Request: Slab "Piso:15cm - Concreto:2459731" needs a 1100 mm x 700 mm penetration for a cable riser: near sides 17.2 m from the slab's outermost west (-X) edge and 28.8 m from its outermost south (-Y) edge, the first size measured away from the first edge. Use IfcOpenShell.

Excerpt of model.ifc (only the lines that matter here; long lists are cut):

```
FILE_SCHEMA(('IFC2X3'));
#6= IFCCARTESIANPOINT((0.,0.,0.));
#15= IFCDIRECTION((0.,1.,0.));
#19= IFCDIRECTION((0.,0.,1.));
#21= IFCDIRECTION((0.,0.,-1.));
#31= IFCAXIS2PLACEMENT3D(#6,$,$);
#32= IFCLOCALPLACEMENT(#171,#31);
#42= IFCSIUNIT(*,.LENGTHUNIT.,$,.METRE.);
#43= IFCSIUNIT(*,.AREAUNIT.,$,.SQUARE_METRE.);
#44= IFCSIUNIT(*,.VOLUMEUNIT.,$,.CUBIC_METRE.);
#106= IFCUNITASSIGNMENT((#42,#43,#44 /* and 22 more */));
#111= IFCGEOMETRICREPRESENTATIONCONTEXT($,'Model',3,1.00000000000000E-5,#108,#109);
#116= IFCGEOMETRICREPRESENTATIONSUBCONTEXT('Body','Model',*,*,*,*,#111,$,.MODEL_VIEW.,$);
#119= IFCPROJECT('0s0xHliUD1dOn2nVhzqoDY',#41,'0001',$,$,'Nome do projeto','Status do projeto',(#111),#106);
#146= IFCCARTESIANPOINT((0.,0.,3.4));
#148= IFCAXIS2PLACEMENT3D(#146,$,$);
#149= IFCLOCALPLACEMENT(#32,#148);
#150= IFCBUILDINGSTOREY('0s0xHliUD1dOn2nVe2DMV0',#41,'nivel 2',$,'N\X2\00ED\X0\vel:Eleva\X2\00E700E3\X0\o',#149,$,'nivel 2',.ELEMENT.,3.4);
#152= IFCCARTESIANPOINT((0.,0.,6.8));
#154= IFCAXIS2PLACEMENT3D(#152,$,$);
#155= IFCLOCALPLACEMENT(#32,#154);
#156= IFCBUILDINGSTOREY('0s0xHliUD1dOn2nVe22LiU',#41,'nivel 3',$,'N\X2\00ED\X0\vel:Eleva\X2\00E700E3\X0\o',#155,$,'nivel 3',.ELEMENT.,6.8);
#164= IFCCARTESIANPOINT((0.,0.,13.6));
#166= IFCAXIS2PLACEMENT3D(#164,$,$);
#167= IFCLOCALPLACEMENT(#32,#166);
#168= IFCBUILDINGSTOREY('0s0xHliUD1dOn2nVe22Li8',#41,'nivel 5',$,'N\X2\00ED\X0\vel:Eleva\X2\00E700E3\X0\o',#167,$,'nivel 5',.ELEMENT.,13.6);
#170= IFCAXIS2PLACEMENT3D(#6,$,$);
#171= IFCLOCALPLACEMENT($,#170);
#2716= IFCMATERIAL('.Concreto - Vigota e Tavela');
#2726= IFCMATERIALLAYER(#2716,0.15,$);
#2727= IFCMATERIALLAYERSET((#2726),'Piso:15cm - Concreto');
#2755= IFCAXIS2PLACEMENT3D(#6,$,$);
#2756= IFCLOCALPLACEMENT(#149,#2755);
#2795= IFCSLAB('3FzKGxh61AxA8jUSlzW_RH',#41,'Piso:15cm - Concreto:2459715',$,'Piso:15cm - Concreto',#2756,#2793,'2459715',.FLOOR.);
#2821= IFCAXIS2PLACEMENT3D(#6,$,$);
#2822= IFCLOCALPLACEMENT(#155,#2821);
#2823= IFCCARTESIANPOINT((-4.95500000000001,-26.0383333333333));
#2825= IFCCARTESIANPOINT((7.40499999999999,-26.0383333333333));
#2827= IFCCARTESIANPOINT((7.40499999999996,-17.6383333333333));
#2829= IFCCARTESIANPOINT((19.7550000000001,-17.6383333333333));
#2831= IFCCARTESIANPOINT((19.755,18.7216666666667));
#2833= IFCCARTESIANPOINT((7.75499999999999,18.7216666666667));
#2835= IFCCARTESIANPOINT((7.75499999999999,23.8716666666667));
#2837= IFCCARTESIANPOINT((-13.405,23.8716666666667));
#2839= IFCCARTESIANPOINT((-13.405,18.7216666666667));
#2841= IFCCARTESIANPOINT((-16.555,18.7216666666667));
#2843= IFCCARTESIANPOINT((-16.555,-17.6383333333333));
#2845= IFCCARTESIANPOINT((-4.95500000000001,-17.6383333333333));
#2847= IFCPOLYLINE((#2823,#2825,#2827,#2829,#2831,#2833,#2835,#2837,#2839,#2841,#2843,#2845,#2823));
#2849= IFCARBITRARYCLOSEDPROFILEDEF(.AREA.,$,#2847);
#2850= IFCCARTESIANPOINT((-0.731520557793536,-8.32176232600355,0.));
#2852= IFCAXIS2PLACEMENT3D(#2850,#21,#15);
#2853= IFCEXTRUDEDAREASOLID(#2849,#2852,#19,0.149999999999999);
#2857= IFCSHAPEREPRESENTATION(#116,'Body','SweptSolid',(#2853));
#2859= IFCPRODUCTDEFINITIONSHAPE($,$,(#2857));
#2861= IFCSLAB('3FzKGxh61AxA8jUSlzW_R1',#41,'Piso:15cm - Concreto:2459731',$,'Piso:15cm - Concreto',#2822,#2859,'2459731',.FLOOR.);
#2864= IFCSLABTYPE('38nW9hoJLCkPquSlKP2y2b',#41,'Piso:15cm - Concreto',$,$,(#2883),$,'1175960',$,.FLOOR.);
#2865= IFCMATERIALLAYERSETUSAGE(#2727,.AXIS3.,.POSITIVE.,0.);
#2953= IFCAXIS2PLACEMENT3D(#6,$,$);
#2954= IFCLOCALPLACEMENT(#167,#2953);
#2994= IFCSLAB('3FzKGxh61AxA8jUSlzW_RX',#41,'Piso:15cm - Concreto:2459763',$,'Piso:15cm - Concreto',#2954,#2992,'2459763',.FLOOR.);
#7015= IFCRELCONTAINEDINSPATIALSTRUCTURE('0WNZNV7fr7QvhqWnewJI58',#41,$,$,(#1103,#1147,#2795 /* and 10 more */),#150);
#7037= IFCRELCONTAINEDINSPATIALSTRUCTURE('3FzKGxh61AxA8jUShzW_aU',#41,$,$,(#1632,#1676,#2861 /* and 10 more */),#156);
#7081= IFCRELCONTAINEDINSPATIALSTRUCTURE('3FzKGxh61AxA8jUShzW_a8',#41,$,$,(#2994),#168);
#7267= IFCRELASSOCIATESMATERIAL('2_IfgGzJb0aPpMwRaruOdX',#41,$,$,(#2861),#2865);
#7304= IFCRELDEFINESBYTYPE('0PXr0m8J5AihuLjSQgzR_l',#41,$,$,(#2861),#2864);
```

```python
import numpy as np
import ifcopenshell
import ifcopenshell.api.feature
import ifcopenshell.api.geometry
import ifcopenshell.api.root
import ifcopenshell.geom
import ifcopenshell.util.placement
import ifcopenshell.util.representation
import ifcopenshell.util.shape
import ifcopenshell.util.unit

model = ifcopenshell.open("model.ifc")
unit_scale = ifcopenshell.util.unit.calculate_unit_scale(model)
settings = ifcopenshell.geom.settings()


def volume(element):
    """Net volume in cubic metres, openings subtracted."""
    shape = ifcopenshell.geom.create_shape(settings, element)
    return ifcopenshell.util.shape.get_volume(shape.geometry)


slab = model.by_guid("3FzKGxh61AxA8jUSlzW_R1")
before = volume(slab)

# Extent in the slab's own axes, in metres. The edges named are its -X and -Y sides.
slab_shape = ifcopenshell.geom.create_shape(settings, slab)
vertices = ifcopenshell.util.shape.get_vertices(slab_shape.geometry)
x_min, y_min, bottom = vertices.min(axis=0)
top = vertices[:, 2].max()

opening = ifcopenshell.api.root.create_entity(model, ifc_class="IfcOpeningElement", name="Cable riser opening")
context = ifcopenshell.util.representation.get_context(model, "Model", "Body", "MODEL_VIEW")
width, depth = 1.1, 0.7
outline = [(0.0, 0.0), (width, 0.0), (width, depth), (0.0, depth), (0.0, 0.0)]
# Overshoot both faces by 50 mm so the cut is clean.
shape = ifcopenshell.api.geometry.add_slab_representation(
    model, context=context, depth=top - bottom + 0.1, polyline=outline
)
ifcopenshell.api.geometry.assign_representation(model, product=opening, representation=shape)

matrix = ifcopenshell.util.placement.get_local_placement(slab.ObjectPlacement)
matrix[:, 3] = matrix @ np.append(np.array([x_min + 17.2, y_min + 28.8, bottom - 0.05]) / unit_scale, 1.0)
ifcopenshell.api.geometry.edit_object_placement(model, product=opening, matrix=matrix, is_si=False)
ifcopenshell.api.feature.add_feature(model, feature=opening, element=slab)

after = volume(slab)

print(f"slab volume {before:.3f} -> {after:.3f} m3")

model.write("model-out.ifc")
```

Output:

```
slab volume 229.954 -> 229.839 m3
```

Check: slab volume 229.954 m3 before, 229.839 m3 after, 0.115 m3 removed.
